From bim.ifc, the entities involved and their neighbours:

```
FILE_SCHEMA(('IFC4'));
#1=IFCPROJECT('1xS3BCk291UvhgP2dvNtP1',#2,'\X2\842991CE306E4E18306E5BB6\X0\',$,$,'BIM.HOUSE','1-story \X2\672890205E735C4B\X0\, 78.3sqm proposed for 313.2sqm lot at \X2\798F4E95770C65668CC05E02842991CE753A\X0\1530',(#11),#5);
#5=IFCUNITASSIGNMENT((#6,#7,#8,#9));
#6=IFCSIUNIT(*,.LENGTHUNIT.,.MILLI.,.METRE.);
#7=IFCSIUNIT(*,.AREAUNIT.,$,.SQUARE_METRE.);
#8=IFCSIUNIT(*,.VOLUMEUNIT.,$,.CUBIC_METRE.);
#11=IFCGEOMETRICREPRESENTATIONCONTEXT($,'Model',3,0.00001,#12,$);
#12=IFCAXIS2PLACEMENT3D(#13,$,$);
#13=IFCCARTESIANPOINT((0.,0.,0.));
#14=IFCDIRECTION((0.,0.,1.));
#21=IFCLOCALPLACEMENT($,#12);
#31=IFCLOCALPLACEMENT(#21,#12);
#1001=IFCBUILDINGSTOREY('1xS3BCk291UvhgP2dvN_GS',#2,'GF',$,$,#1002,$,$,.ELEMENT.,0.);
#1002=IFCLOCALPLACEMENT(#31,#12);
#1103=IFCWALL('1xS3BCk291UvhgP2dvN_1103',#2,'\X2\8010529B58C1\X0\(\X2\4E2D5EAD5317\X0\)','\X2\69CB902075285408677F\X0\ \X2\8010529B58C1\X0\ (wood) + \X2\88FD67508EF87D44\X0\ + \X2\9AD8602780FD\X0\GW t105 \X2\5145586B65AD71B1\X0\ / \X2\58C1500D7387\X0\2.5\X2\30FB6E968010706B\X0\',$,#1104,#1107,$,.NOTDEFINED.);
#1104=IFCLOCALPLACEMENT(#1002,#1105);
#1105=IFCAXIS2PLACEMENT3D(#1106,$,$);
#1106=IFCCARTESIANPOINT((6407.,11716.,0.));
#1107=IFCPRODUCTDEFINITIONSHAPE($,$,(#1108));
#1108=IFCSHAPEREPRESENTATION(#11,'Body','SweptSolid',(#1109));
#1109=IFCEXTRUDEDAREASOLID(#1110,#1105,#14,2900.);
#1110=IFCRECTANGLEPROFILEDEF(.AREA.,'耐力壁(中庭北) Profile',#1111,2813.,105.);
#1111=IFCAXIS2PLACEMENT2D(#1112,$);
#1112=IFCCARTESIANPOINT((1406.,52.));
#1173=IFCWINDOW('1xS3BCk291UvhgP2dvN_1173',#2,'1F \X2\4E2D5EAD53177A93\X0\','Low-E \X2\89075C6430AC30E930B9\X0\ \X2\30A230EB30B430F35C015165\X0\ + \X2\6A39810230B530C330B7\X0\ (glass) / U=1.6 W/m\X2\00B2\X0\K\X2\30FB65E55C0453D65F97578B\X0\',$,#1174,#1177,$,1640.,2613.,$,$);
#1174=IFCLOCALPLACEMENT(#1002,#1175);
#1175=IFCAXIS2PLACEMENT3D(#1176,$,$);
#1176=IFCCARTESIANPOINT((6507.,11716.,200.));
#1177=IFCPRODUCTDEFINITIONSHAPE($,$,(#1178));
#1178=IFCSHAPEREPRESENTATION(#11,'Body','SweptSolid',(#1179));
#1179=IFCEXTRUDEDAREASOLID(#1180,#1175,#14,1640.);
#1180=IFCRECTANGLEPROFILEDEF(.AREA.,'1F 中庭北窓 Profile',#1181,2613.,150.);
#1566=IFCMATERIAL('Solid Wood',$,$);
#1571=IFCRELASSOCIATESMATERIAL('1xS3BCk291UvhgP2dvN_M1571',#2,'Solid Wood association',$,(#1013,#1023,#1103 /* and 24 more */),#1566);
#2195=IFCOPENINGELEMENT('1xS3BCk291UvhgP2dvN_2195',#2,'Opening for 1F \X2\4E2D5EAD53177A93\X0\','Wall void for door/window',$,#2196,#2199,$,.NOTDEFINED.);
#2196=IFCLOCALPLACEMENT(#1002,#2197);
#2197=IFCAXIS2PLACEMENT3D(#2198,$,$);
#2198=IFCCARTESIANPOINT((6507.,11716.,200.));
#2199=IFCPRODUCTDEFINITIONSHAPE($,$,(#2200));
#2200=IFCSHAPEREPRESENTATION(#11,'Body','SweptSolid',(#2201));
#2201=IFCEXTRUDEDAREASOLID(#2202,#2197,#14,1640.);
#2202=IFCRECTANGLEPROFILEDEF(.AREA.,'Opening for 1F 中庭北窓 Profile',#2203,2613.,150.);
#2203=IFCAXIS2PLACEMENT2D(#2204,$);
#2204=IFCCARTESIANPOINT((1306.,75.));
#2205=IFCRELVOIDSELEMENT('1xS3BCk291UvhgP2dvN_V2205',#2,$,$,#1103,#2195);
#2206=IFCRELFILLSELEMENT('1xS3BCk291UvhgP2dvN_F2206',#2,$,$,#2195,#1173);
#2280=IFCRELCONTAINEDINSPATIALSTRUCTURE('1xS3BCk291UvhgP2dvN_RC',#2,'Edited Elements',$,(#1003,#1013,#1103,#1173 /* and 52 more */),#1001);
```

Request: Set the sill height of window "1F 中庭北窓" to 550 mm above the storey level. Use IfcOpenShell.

```python
import numpy as np
import ifcopenshell
import ifcopenshell.api.geometry
import ifcopenshell.geom
import ifcopenshell.util.element
import ifcopenshell.util.placement
import ifcopenshell.util.shape
import ifcopenshell.util.unit

model = ifcopenshell.open("bim.ifc")
unit_scale = ifcopenshell.util.unit.calculate_unit_scale(model)

window = model.by_guid("1xS3BCk291UvhgP2dvN_1173")
opening = window.FillsVoids[0].RelatingOpeningElement
storey = ifcopenshell.util.element.get_container(window, ifc_class="IfcBuildingStorey")
level = ifcopenshell.util.placement.get_local_placement(storey.ObjectPlacement)[2, 3]

# The opening's origin need not be at the sill, so measure its lowest point.
shape = ifcopenshell.geom.create_shape(ifcopenshell.geom.settings(), opening)
bottom = ifcopenshell.util.shape.get_shape_bottom_elevation(shape, shape.geometry) / unit_scale
dz = level + 550.0 - bottom

shift = np.array([0.0, 0.0, dz])
# The window is not placed relative to its opening, so move both.
for product in (opening, window):
    matrix = ifcopenshell.util.placement.get_local_placement(product.ObjectPlacement)
    matrix[:3, 3] += shift
    ifcopenshell.api.geometry.edit_object_placement(model, product=product, matrix=matrix, is_si=False)

print(f"moved by {dz * unit_scale:+.3f} m")

model.write("bim_updated.ifc")
```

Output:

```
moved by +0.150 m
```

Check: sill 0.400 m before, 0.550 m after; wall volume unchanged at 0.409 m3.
